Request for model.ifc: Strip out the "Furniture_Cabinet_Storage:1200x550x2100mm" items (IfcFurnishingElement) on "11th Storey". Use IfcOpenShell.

First a look at what the model holds.

```python
import ifcopenshell
import ifcopenshell.util.element

model = ifcopenshell.open("model.ifc")
print(model.schema)
storey = next(s for s in model.by_type("IfcBuildingStorey") if s.Name == "11th Storey")
furniture = [e for e in ifcopenshell.util.element.get_decomposition(storey) if e.is_a("IfcFurnishingElement")]
seen = {}
for e in furniture:
    element_type = ifcopenshell.util.element.get_type(e)
    name = element_type.Name if element_type not in (None, e) else None
    seen[name] = seen.get(name, 0) + 1
for name, count in sorted(seen.items(), key=str):
    print(count, "x", name)
```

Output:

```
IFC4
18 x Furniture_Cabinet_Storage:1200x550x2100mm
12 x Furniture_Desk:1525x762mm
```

```python
import ifcopenshell
import ifcopenshell.api.root
import ifcopenshell.util.element

model = ifcopenshell.open("model.ifc")

storey = next(s for s in model.by_type("IfcBuildingStorey") if s.Name == "11th Storey")
furniture = [e for e in ifcopenshell.util.element.get_decomposition(storey) if e.is_a("IfcFurnishingElement")]
targets = [e for e in furniture if (t := ifcopenshell.util.element.get_type(e)) not in (None, e) and t.Name == "Furniture_Cabinet_Storage:1200x550x2100mm"]

for e in targets:
    ifcopenshell.api.root.remove_product(model, product=e)
print(len(targets), "removed")

model.write("model_v2.ifc")
```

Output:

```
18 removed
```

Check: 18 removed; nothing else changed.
